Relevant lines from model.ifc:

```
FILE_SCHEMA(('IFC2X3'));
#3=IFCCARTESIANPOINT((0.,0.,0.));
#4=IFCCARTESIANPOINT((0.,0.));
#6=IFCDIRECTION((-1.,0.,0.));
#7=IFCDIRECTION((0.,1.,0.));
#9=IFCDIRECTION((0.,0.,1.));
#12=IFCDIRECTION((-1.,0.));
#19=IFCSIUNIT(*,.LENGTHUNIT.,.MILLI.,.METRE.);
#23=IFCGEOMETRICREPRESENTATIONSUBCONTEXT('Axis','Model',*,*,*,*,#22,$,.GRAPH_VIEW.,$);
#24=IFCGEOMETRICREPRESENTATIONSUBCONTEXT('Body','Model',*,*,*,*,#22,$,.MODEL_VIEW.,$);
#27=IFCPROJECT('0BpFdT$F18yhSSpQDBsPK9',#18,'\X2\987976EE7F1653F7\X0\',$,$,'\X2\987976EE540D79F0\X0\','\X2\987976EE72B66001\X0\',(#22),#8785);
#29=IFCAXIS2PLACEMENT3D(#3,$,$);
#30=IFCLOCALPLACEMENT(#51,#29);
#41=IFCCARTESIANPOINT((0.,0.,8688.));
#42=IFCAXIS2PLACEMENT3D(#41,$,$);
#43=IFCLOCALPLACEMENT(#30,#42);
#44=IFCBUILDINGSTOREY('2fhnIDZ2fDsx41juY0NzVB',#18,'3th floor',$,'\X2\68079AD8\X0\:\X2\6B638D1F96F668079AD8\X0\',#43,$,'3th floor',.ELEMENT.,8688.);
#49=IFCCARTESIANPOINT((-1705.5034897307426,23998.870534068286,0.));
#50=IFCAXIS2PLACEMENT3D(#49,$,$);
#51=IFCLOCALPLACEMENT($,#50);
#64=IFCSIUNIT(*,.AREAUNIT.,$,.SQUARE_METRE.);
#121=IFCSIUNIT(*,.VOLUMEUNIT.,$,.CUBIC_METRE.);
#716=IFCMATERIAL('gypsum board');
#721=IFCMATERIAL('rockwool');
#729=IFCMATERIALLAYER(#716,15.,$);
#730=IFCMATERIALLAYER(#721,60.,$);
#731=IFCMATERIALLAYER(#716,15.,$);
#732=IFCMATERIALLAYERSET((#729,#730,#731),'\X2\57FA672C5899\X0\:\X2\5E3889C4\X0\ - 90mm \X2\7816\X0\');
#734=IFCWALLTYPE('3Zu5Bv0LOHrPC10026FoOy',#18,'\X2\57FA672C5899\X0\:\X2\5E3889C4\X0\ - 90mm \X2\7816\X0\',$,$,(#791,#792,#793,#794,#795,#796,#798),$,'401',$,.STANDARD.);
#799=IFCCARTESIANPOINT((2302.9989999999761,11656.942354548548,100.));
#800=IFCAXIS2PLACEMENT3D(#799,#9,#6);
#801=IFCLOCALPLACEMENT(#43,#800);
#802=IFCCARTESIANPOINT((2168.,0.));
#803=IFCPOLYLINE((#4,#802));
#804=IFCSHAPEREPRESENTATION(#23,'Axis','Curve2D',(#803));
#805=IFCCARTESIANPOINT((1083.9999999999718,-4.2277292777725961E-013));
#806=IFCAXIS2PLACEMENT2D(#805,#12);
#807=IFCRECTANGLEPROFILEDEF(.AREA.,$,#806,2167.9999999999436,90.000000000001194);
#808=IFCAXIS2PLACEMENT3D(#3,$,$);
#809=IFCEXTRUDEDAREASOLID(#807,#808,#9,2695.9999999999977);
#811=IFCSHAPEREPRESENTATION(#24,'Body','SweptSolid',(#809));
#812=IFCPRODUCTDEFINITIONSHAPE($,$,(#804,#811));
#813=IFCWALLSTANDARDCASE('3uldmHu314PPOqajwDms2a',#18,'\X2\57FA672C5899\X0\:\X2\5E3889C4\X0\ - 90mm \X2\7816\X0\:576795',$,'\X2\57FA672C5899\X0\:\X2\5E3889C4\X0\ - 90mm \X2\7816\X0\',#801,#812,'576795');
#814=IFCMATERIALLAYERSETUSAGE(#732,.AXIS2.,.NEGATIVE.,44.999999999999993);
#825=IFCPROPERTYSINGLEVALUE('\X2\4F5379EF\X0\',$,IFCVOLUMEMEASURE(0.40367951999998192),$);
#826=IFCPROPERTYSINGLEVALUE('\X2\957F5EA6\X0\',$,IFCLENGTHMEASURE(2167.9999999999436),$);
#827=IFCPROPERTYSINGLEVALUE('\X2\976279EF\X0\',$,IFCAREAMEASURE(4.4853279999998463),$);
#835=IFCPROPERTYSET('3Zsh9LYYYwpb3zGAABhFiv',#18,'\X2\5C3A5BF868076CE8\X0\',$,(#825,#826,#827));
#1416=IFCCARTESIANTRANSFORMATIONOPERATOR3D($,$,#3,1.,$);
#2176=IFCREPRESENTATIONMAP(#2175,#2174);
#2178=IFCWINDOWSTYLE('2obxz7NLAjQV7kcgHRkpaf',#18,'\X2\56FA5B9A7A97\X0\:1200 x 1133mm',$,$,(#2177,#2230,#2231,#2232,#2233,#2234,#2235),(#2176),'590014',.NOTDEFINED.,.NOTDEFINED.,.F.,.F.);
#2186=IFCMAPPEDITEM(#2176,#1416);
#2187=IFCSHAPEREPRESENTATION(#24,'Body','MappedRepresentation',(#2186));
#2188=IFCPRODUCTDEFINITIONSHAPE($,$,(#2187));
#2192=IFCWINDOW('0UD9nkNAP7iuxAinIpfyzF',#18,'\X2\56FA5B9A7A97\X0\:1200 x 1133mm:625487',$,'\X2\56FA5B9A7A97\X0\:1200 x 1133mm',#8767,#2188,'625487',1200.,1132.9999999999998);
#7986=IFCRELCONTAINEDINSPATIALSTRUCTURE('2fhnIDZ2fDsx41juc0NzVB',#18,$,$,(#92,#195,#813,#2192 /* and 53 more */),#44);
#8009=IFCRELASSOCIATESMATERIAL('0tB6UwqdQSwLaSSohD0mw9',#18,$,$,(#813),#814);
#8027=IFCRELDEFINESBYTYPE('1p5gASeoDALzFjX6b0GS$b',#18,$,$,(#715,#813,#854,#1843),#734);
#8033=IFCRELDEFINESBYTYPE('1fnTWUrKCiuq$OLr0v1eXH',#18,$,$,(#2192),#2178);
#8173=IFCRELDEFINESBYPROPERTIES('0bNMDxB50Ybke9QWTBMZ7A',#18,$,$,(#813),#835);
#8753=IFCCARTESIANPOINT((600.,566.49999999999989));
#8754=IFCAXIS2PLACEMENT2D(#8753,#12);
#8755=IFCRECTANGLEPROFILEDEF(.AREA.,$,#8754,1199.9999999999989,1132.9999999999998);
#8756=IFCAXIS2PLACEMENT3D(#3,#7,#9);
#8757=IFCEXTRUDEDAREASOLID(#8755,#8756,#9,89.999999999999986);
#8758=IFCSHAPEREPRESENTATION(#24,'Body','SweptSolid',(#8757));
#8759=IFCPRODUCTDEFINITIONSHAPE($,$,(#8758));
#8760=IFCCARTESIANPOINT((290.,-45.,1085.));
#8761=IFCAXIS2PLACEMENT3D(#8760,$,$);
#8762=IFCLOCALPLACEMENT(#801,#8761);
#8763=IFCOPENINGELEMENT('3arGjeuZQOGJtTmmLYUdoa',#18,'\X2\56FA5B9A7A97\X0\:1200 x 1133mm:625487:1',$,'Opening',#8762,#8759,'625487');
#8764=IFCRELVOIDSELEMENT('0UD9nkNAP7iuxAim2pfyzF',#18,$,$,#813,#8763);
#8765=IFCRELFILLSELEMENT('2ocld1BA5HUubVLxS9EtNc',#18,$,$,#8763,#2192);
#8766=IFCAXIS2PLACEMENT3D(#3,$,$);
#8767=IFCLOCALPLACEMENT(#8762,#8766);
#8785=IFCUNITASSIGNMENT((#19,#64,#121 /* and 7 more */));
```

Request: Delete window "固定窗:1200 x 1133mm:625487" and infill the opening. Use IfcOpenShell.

```python
import ifcopenshell
import ifcopenshell.api.feature
import ifcopenshell.api.pset
import ifcopenshell.api.root
import ifcopenshell.geom
import ifcopenshell.util.element
import ifcopenshell.util.shape
import ifcopenshell.util.unit

model = ifcopenshell.open("model.ifc")
area_scale = ifcopenshell.util.unit.calculate_unit_scale(model, "AREAUNIT")
volume_scale = ifcopenshell.util.unit.calculate_unit_scale(model, "VOLUMEUNIT")
settings = ifcopenshell.geom.settings()


def volume(element):
    """Net volume in cubic metres, openings subtracted."""
    shape = ifcopenshell.geom.create_shape(settings, element)
    return ifcopenshell.util.shape.get_volume(shape.geometry)


window = model.by_guid("0UD9nkNAP7iuxAinIpfyzF")
opening = window.FillsVoids[0].RelatingOpeningElement
wall = opening.VoidsElements[0].RelatingBuildingElement
before = volume(wall)

ifcopenshell.api.root.remove_product(model, product=window)
ifcopenshell.api.feature.remove_feature(model, feature=opening)

after = volume(wall)
thickness = 0.09  # wall thickness in metres

# Update the wall's stored quantities.
pset = model.by_id(ifcopenshell.util.element.get_pset(wall, "尺寸标注", should_inherit=False)["id"])
ifcopenshell.api.pset.edit_pset(model, pset=pset, properties={
    "体积": model.create_entity("IfcVolumeMeasure", after / volume_scale),
    "面积": model.create_entity("IfcAreaMeasure", after / thickness / area_scale),
})

print(f"wall volume {before:.3f} -> {after:.3f} m3")

model.write("model_v2.ifc")
```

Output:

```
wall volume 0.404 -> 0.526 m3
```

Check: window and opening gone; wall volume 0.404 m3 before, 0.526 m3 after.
